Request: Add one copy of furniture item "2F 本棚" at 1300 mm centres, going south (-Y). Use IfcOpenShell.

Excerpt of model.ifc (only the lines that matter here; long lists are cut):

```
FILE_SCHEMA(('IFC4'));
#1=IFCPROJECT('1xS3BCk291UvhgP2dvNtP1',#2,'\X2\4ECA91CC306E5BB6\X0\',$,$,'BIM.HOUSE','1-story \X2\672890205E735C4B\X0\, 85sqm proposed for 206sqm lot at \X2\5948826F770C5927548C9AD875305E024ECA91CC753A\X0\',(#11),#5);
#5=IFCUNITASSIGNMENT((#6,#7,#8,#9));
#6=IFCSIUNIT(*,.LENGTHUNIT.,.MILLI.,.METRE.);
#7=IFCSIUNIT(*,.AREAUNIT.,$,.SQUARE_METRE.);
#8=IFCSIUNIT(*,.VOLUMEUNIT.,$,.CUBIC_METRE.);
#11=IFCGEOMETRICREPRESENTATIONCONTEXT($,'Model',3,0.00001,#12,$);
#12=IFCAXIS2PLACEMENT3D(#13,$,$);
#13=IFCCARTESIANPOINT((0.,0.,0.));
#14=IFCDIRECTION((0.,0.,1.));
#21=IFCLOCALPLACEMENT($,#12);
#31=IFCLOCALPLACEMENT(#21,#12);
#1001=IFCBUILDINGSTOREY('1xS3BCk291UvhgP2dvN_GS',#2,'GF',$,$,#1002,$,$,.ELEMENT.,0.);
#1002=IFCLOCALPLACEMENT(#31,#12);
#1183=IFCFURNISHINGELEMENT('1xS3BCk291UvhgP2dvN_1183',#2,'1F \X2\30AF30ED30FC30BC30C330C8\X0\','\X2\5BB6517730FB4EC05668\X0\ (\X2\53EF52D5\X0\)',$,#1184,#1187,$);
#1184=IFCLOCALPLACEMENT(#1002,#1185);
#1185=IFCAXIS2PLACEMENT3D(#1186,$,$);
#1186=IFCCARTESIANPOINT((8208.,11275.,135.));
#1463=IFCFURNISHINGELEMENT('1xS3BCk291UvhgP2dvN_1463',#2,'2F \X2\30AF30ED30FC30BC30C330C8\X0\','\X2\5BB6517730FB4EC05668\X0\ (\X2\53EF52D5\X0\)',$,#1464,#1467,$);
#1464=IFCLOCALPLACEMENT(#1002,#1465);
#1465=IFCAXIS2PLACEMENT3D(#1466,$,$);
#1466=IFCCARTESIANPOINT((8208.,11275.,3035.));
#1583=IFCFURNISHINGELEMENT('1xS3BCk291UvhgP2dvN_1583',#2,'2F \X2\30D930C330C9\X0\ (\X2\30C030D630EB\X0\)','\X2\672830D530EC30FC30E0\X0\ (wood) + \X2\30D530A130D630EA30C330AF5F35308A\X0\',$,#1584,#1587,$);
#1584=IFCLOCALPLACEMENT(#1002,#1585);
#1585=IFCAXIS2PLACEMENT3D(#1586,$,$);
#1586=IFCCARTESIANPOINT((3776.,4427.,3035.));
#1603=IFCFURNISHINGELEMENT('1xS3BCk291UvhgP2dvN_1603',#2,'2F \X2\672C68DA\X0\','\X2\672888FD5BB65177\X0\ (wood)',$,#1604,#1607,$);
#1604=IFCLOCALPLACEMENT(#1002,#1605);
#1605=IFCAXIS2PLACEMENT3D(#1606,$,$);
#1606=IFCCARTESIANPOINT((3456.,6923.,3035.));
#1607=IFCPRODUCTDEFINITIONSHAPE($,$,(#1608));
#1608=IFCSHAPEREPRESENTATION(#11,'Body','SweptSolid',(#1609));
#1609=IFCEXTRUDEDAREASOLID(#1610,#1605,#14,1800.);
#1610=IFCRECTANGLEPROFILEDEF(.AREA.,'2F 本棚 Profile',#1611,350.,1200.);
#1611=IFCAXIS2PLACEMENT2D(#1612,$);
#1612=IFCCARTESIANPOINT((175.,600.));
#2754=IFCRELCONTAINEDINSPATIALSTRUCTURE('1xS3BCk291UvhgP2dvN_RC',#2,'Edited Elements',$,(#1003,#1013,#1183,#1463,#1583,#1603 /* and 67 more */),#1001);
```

```python
import numpy as np
import ifcopenshell
import ifcopenshell.api.geometry
import ifcopenshell.api.root
import ifcopenshell.util.element
import ifcopenshell.util.placement
import ifcopenshell.util.unit

model = ifcopenshell.open("model.ifc")
unit_scale = ifcopenshell.util.unit.calculate_unit_scale(model)


def reuse_history(source, copy):
    """copy_class also copies each property set's owner history, people and application; keep the originals."""
    for rel in copy.IsDefinedBy:
        if rel.is_a("IfcRelDefinesByProperties") and (history := rel.RelatingPropertyDefinition.OwnerHistory):
            rel.RelatingPropertyDefinition.OwnerHistory = source.OwnerHistory
            ifcopenshell.util.element.remove_deep2(model, history)


source = model.by_guid("1xS3BCk291UvhgP2dvN_1603")
base = ifcopenshell.util.placement.get_local_placement(source.ObjectPlacement)
step = np.array([0.0, -1.0, 0.0]) * 1.3 / unit_scale

for i in range(1, 2):
    copy = ifcopenshell.api.root.copy_class(model, product=source)
    copy.Representation = ifcopenshell.util.element.copy_deep(
        model, source.Representation, exclude=["IfcGeometricRepresentationContext", "IfcRepresentationMap"]
    )
    reuse_history(source, copy)
    matrix = base.copy()
    matrix[:3, 3] += i * step
    print("added at", matrix[:3, 3].round(3) + 0.0)
    ifcopenshell.api.geometry.edit_object_placement(model, product=copy, matrix=matrix, is_si=False)

model.write("model_updated.ifc")
```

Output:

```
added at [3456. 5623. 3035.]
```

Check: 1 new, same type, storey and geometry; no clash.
